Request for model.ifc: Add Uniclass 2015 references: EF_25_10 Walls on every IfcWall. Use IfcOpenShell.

First a look at what the model holds.

```python
import ifcopenshell

model = ifcopenshell.open("model.ifc")
print(model.schema)
print("classifications:", [c.Name for c in model.by_type("IfcClassification")])
for ifc_class in ("IfcDoor", "IfcRoof", "IfcStair", "IfcWall", "IfcWindow"):
    print(ifc_class, len(model.by_type(ifc_class)))
```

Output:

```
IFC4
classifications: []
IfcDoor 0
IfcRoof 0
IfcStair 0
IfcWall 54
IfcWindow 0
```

```python
import ifcopenshell
import ifcopenshell.api.classification

model = ifcopenshell.open("model.ifc")

system = ifcopenshell.api.classification.add_classification(model, classification="Uniclass 2015")

codes = {
    "IfcWall": ("EF_25_10", "Walls"),
}
for ifc_class, (code, name) in codes.items():
    products = model.by_type(ifc_class)
    ifcopenshell.api.classification.add_reference(
        model, products=products, classification=system, identification=code, name=name
    )
    print(code, len(products))

model.write("model_updated.ifc")
```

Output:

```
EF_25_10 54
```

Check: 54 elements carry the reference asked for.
